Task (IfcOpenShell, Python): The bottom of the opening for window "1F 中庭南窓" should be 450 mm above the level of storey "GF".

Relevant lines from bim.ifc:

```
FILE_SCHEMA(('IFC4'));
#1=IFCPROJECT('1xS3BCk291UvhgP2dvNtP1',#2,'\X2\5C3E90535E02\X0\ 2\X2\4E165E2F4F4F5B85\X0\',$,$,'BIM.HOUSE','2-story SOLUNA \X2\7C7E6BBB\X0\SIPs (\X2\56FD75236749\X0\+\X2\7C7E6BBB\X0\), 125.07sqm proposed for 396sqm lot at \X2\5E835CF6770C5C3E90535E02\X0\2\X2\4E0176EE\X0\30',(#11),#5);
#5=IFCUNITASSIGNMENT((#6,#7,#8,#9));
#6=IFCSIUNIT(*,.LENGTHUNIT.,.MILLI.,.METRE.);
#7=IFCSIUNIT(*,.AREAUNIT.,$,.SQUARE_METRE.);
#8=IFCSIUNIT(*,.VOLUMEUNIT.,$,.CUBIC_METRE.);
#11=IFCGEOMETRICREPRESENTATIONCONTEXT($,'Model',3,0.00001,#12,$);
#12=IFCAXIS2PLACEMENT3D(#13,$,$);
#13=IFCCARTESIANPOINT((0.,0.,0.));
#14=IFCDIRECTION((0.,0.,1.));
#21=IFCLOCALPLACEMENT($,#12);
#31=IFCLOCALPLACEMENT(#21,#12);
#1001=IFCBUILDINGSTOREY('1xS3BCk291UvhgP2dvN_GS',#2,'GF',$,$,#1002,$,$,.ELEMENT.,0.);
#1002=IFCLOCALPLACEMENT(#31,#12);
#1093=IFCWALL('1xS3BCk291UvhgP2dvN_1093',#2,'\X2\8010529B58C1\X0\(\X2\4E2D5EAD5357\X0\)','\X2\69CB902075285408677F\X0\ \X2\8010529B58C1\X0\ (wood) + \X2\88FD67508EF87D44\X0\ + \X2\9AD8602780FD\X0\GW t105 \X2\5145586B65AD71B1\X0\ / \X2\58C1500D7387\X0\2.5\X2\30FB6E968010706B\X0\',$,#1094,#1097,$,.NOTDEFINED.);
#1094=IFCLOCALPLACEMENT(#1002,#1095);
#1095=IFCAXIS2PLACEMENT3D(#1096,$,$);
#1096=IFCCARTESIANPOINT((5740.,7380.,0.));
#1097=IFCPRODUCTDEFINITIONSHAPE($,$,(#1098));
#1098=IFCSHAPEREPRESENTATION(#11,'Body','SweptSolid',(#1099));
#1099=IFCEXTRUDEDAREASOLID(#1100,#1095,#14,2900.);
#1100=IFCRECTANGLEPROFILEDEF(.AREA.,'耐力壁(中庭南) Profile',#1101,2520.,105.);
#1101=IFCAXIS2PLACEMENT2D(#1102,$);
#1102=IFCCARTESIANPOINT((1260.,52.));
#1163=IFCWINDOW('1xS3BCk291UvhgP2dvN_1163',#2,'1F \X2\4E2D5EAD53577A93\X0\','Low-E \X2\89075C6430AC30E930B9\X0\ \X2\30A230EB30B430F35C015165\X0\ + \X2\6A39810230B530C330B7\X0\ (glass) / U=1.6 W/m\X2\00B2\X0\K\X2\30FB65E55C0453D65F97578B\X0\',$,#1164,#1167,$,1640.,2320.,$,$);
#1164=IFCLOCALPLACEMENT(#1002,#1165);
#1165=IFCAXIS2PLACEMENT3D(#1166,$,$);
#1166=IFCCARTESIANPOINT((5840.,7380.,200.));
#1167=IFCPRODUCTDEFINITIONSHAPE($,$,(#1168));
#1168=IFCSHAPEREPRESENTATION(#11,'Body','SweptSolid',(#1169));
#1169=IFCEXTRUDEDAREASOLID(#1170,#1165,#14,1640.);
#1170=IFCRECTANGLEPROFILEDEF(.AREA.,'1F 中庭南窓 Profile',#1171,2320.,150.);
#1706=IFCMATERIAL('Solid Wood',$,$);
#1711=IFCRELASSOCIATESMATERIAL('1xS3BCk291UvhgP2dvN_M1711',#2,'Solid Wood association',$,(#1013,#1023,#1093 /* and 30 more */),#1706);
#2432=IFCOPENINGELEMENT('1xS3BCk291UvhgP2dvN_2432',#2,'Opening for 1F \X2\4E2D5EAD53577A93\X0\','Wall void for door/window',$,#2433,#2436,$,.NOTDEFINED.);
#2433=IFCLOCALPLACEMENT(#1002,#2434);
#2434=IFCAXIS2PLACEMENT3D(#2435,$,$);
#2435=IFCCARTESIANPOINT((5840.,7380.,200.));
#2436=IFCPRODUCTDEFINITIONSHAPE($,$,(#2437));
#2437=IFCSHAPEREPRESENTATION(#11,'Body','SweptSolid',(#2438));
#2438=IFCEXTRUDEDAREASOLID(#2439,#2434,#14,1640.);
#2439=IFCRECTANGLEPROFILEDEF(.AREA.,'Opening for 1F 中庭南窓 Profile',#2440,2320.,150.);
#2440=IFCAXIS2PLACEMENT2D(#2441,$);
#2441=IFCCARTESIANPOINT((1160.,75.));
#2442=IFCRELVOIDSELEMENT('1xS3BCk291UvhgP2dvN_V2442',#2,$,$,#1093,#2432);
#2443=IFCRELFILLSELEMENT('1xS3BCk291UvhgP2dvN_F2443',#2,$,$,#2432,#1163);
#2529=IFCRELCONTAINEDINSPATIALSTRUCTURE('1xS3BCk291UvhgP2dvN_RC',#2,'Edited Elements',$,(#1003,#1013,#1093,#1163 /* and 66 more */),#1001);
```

```python
import numpy as np
import ifcopenshell
import ifcopenshell.api.geometry
import ifcopenshell.geom
import ifcopenshell.util.element
import ifcopenshell.util.placement
import ifcopenshell.util.shape
import ifcopenshell.util.unit

model = ifcopenshell.open("bim.ifc")
unit_scale = ifcopenshell.util.unit.calculate_unit_scale(model)

window = model.by_guid("1xS3BCk291UvhgP2dvN_1163")
opening = window.FillsVoids[0].RelatingOpeningElement
storey = ifcopenshell.util.element.get_container(window, ifc_class="IfcBuildingStorey")
level = ifcopenshell.util.placement.get_local_placement(storey.ObjectPlacement)[2, 3]

# The opening's origin need not be at the sill, so measure its lowest point.
shape = ifcopenshell.geom.create_shape(ifcopenshell.geom.settings(), opening)
bottom = ifcopenshell.util.shape.get_shape_bottom_elevation(shape, shape.geometry) / unit_scale
dz = level + 450.0 - bottom

shift = np.array([0.0, 0.0, dz])
# The window is not placed relative to its opening, so move both.
for product in (opening, window):
    matrix = ifcopenshell.util.placement.get_local_placement(product.ObjectPlacement)
    matrix[:3, 3] += shift
    ifcopenshell.api.geometry.edit_object_placement(model, product=product, matrix=matrix, is_si=False)

print(f"moved by {dz * unit_scale:+.3f} m")

model.write("bim_v2.ifc")
```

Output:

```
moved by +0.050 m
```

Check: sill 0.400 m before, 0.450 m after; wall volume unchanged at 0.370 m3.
